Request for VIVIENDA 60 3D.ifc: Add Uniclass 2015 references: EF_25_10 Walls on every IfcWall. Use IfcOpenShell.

First a look at what the model holds.

```python
import ifcopenshell

model = ifcopenshell.open("VIVIENDA 60 3D.ifc")
print(model.schema)
print("classifications:", [c.Name for c in model.by_type("IfcClassification")])
for ifc_class in ("IfcDoor", "IfcRoof", "IfcStair", "IfcWall", "IfcWindow"):
    print(ifc_class, len(model.by_type(ifc_class)))
```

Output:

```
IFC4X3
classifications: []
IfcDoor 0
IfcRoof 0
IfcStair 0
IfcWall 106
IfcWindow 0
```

```python
import ifcopenshell
import ifcopenshell.api.classification

model = ifcopenshell.open("VIVIENDA 60 3D.ifc")

system = ifcopenshell.api.classification.add_classification(model, classification="Uniclass 2015")

codes = {
    "IfcWall": ("EF_25_10", "Walls"),
}
for ifc_class, (code, name) in codes.items():
    products = model.by_type(ifc_class)
    ifcopenshell.api.classification.add_reference(
        model, products=products, classification=system, identification=code, name=name
    )
    print(code, len(products))

model.write("VIVIENDA 60 3D_v2.ifc")
```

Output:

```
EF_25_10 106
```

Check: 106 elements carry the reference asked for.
